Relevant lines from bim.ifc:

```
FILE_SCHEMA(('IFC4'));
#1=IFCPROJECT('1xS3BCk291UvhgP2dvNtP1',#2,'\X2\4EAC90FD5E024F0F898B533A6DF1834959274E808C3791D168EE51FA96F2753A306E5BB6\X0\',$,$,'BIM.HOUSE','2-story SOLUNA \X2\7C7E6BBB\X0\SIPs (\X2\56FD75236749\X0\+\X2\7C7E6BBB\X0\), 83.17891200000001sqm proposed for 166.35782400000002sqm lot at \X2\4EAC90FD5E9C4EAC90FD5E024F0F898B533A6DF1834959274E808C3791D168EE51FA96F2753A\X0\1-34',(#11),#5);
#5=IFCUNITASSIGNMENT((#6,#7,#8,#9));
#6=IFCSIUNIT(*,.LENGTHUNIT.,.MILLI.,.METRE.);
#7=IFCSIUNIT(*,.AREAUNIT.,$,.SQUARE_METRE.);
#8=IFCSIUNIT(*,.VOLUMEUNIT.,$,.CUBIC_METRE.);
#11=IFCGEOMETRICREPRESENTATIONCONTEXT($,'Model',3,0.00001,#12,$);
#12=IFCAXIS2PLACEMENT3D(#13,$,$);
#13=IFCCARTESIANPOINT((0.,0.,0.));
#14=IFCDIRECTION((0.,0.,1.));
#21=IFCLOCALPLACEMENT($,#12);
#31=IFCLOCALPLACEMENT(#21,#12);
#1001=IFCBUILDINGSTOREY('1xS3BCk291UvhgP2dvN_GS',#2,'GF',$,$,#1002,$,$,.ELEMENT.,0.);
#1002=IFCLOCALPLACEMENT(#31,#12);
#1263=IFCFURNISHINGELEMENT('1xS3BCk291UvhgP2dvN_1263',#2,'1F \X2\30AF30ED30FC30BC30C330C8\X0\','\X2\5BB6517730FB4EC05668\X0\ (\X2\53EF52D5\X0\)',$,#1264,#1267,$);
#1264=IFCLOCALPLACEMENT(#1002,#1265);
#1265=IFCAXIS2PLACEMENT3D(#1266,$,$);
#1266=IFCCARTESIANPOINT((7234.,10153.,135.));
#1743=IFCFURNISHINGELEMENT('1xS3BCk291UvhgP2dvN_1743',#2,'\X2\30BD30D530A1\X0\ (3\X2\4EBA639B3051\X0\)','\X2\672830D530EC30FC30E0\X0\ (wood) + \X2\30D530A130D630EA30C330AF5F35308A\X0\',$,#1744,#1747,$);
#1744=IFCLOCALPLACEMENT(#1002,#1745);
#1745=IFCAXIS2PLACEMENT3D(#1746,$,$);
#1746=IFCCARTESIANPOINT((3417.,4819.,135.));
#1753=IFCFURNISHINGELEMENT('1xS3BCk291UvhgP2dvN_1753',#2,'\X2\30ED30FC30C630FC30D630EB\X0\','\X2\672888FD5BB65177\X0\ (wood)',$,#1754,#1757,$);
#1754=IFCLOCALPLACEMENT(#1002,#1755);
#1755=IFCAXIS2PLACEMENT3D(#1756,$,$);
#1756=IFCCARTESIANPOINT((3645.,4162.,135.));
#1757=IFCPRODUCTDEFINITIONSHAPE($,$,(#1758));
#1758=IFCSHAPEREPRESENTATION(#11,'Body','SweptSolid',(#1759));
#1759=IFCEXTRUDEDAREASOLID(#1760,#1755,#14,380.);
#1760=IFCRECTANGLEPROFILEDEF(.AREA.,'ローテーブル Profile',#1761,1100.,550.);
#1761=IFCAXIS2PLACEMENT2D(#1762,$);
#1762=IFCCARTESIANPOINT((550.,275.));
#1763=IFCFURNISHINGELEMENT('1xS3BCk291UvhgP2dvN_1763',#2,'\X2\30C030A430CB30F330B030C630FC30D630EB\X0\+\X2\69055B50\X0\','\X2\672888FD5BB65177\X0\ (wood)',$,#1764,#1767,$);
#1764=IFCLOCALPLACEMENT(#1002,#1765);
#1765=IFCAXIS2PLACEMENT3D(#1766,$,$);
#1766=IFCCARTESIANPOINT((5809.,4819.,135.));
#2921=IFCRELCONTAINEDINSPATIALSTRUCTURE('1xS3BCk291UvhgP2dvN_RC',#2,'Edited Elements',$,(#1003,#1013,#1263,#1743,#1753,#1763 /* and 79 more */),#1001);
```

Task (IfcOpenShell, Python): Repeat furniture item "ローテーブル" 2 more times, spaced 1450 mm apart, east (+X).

```python
import numpy as np
import ifcopenshell
import ifcopenshell.api.geometry
import ifcopenshell.api.root
import ifcopenshell.util.element
import ifcopenshell.util.placement

model = ifcopenshell.open("bim.ifc")


def reuse_history(source, copy):
    """copy_class also copies each property set's owner history, people and application; keep the originals."""
    for rel in copy.IsDefinedBy:
        if rel.is_a("IfcRelDefinesByProperties") and (history := rel.RelatingPropertyDefinition.OwnerHistory):
            rel.RelatingPropertyDefinition.OwnerHistory = source.OwnerHistory
            ifcopenshell.util.element.remove_deep2(model, history)


source = model.by_guid("1xS3BCk291UvhgP2dvN_1753")
base = ifcopenshell.util.placement.get_local_placement(source.ObjectPlacement)
step = np.array([1.0, 0.0, 0.0]) * 1450.0

for i in range(1, 3):
    copy = ifcopenshell.api.root.copy_class(model, product=source)
    copy.Representation = ifcopenshell.util.element.copy_deep(
        model, source.Representation, exclude=["IfcGeometricRepresentationContext", "IfcRepresentationMap"]
    )
    reuse_history(source, copy)
    matrix = base.copy()
    matrix[:3, 3] += i * step
    print("added at", matrix[:3, 3].round(3) + 0.0)
    ifcopenshell.api.geometry.edit_object_placement(model, product=copy, matrix=matrix, is_si=False)

model.write("bim_rev.ifc")
```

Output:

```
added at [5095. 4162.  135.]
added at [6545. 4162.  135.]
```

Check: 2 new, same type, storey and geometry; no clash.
